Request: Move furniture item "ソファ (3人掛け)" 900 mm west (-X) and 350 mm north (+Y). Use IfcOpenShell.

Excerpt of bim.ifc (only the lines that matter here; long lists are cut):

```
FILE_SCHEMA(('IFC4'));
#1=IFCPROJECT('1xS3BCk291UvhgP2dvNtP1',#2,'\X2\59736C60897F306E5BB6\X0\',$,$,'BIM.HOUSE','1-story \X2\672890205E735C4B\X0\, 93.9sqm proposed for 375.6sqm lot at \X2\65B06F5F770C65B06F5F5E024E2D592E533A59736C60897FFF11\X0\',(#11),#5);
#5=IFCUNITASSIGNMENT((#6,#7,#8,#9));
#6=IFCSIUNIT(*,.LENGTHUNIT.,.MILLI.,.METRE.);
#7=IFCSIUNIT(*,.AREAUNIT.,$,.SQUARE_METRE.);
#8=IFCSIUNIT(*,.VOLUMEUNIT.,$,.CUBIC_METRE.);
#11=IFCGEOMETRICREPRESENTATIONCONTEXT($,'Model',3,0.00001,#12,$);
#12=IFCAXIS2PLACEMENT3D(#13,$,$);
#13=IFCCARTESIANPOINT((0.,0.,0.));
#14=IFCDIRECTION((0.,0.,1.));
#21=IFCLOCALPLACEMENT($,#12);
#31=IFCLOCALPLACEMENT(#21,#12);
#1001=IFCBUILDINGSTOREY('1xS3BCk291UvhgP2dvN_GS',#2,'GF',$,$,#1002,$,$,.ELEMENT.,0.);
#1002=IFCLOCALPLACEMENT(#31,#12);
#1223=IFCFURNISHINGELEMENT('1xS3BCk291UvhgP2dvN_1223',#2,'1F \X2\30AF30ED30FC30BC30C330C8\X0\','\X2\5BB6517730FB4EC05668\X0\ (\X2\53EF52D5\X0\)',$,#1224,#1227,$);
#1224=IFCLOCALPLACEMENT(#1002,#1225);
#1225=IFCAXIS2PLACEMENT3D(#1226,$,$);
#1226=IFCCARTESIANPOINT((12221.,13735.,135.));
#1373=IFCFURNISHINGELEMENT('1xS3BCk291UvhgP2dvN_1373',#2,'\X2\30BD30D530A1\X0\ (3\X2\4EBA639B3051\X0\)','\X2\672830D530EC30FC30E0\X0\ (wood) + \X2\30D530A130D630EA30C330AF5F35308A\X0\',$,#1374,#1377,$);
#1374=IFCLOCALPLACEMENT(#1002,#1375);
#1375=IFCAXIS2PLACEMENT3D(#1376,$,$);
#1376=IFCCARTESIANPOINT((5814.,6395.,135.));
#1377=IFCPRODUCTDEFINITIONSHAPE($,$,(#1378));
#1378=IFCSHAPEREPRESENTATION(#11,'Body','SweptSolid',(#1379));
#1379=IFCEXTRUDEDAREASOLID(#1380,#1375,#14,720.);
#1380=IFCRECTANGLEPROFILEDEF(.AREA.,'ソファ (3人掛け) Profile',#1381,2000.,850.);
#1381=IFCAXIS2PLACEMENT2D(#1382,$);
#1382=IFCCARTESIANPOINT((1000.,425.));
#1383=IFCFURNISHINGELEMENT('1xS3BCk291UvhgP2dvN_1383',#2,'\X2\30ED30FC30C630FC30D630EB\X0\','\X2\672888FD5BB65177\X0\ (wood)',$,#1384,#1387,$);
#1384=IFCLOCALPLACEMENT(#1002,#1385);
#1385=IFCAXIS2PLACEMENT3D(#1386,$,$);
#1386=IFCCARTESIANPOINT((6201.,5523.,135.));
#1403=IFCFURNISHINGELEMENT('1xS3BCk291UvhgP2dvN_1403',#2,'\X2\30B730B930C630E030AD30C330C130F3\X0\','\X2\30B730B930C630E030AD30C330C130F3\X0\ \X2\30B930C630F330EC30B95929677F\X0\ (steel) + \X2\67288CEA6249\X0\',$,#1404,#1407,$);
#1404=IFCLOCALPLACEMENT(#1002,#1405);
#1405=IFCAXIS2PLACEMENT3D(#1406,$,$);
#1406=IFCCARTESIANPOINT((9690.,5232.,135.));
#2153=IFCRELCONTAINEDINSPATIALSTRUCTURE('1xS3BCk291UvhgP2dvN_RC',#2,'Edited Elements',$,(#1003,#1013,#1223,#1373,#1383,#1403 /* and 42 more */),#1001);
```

```python
import ifcopenshell
import ifcopenshell.api.geometry
import ifcopenshell.util.placement
import ifcopenshell.util.unit

model = ifcopenshell.open("bim.ifc")
unit_scale = ifcopenshell.util.unit.calculate_unit_scale(model)

item = model.by_id(1373)
matrix = ifcopenshell.util.placement.get_local_placement(item.ObjectPlacement)
matrix[0, 3] -= 0.9 / unit_scale
matrix[1, 3] += 0.35 / unit_scale
ifcopenshell.api.geometry.edit_object_placement(model, product=item, matrix=matrix, is_si=False)

print(ifcopenshell.util.placement.get_local_placement(item.ObjectPlacement).round(3) + 0.0)

model.write("bim_rev.ifc")
```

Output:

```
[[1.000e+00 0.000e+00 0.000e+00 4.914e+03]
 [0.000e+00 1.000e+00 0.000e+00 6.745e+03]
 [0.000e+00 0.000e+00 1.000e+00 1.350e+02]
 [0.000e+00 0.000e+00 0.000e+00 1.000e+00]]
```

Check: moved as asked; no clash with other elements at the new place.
